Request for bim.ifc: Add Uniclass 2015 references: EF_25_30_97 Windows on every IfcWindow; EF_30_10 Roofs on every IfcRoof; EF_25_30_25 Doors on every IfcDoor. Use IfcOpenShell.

First a look at what the model holds.

```python
import ifcopenshell

model = ifcopenshell.open("bim.ifc")
print(model.schema)
print("classifications:", [c.Name for c in model.by_type("IfcClassification")])
for ifc_class in ("IfcDoor", "IfcRoof", "IfcStair", "IfcWall", "IfcWindow"):
    print(ifc_class, len(model.by_type(ifc_class)))
```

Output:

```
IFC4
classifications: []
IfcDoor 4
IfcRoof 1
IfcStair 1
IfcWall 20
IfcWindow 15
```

```python
import ifcopenshell
import ifcopenshell.api.classification

model = ifcopenshell.open("bim.ifc")

system = ifcopenshell.api.classification.add_classification(model, classification="Uniclass 2015")

codes = {
    "IfcWindow": ("EF_25_30_97", "Windows"),
    "IfcRoof": ("EF_30_10", "Roofs"),
    "IfcDoor": ("EF_25_30_25", "Doors"),
}
for ifc_class, (code, name) in codes.items():
    products = model.by_type(ifc_class)
    ifcopenshell.api.classification.add_reference(
        model, products=products, classification=system, identification=code, name=name
    )
    print(code, len(products))

model.write("bim_edited.ifc")
```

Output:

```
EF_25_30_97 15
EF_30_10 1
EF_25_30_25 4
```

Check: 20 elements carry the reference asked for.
